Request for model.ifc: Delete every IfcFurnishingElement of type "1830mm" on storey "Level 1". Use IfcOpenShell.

First a look at what the model holds.

```python
import ifcopenshell
import ifcopenshell.util.element

model = ifcopenshell.open("model.ifc")
print(model.schema)
storey = next(s for s in model.by_type("IfcBuildingStorey") if s.Name == "Level 1")
furniture = [e for e in ifcopenshell.util.element.get_decomposition(storey) if e.is_a("IfcFurnishingElement")]
seen = {}
for e in furniture:
    element_type = ifcopenshell.util.element.get_type(e)
    name = element_type.Name if element_type not in (None, e) else None
    seen[name] = seen.get(name, 0) + 1
for name, count in sorted(seen.items(), key=str):
    print(count, "x", name)
```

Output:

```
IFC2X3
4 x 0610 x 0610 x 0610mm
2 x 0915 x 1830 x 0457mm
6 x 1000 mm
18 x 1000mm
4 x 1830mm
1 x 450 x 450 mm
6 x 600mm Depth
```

```python
import ifcopenshell
import ifcopenshell.api.root
import ifcopenshell.util.element

model = ifcopenshell.open("model.ifc")

storey = next(s for s in model.by_type("IfcBuildingStorey") if s.Name == "Level 1")
furniture = [e for e in ifcopenshell.util.element.get_decomposition(storey) if e.is_a("IfcFurnishingElement")]
targets = [e for e in furniture if (t := ifcopenshell.util.element.get_type(e)) not in (None, e) and t.Name == "1830mm"]

for e in targets:
    ifcopenshell.api.root.remove_product(model, product=e)
print(len(targets), "removed")

model.write("model-out.ifc")
```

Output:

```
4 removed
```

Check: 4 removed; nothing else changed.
